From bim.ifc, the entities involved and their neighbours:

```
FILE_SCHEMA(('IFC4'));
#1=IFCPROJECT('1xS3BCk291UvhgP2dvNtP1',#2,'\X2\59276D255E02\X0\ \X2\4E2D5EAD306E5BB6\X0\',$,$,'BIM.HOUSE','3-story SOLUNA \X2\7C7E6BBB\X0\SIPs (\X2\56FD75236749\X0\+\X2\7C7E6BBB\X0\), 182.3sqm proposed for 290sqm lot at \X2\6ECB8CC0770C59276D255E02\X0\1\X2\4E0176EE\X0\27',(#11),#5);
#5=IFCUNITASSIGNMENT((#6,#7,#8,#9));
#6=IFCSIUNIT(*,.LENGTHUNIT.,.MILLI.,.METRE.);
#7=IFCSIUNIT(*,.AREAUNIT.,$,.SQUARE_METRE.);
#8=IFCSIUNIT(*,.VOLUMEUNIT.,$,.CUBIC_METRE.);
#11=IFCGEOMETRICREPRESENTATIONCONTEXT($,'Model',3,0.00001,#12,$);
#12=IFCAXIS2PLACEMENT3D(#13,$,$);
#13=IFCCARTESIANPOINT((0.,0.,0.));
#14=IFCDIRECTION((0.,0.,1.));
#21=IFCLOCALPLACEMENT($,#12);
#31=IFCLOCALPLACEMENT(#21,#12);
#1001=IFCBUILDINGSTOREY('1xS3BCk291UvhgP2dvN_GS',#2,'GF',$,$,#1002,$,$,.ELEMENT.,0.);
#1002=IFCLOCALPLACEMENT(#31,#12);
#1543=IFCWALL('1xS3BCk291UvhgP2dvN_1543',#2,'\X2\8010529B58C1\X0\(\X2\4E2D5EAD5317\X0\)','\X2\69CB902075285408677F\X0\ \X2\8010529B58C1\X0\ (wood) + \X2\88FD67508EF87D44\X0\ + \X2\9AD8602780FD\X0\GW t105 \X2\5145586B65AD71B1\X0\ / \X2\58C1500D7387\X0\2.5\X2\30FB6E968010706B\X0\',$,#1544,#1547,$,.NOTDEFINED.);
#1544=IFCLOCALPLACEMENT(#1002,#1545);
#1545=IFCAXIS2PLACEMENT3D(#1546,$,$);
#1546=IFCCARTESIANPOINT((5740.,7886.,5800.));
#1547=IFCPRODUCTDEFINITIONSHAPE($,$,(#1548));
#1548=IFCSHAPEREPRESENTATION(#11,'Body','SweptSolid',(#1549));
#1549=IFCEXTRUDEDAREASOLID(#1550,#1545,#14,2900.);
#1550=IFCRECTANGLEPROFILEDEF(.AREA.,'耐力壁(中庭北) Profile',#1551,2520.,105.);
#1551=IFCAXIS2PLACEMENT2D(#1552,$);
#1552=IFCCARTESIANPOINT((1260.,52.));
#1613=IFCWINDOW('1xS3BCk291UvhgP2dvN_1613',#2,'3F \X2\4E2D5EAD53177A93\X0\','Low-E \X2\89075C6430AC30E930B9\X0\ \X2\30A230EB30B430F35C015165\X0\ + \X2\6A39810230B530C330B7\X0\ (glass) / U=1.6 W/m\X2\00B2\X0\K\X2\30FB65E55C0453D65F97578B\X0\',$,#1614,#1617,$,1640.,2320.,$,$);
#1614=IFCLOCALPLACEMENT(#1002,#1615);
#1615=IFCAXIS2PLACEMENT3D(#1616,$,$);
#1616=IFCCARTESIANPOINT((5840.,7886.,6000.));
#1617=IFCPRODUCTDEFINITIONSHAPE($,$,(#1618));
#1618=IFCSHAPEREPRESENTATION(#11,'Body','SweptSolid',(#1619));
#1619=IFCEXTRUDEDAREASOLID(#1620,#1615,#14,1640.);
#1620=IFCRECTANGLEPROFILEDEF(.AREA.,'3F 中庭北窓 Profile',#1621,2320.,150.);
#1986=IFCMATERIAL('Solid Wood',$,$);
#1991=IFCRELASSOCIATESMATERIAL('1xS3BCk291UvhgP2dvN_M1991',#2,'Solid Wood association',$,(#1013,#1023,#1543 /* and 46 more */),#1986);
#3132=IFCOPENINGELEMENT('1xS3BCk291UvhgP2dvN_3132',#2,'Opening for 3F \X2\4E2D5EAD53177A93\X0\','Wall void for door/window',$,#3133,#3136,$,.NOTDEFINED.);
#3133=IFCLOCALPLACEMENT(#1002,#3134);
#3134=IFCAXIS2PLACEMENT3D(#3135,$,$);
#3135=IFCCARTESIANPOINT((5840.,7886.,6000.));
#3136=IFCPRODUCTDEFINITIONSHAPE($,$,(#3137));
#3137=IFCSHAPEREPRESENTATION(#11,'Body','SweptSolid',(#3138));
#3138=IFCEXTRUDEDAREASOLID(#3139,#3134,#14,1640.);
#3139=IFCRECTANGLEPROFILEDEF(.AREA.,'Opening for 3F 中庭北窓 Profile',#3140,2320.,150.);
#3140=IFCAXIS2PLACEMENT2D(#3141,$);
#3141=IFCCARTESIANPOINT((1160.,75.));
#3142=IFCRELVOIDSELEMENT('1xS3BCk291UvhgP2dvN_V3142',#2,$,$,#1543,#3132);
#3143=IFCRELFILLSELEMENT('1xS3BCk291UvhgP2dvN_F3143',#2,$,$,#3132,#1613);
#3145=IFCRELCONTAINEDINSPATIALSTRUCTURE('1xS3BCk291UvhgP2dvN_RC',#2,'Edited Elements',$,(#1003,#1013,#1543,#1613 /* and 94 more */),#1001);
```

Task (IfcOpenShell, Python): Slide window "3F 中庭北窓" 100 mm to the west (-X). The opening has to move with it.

```python
import ifcopenshell
import ifcopenshell.api.geometry
import ifcopenshell.util.placement

model = ifcopenshell.open("bim.ifc")

window = model.by_guid("1xS3BCk291UvhgP2dvN_1613")
opening = window.FillsVoids[0].RelatingOpeningElement
wall = opening.VoidsElements[0].RelatingBuildingElement

wall_matrix = ifcopenshell.util.placement.get_local_placement(wall.ObjectPlacement)
shift = wall_matrix[:3, 0] * -100.0
before = ifcopenshell.util.placement.get_local_placement(window.ObjectPlacement)[:3, 3].copy()

# The window is not placed relative to its opening, so move both.
for product in (opening, window):
    matrix = ifcopenshell.util.placement.get_local_placement(product.ObjectPlacement)
    matrix[:3, 3] += shift
    ifcopenshell.api.geometry.edit_object_placement(model, product=product, matrix=matrix, is_si=False)

after = ifcopenshell.util.placement.get_local_placement(window.ObjectPlacement)[:3, 3]
print("window moved by", (after - before).round(3) + 0.0)

model.write("bim_v2.ifc")
```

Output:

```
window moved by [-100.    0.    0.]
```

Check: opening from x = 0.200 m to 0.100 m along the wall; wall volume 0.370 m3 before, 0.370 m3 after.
